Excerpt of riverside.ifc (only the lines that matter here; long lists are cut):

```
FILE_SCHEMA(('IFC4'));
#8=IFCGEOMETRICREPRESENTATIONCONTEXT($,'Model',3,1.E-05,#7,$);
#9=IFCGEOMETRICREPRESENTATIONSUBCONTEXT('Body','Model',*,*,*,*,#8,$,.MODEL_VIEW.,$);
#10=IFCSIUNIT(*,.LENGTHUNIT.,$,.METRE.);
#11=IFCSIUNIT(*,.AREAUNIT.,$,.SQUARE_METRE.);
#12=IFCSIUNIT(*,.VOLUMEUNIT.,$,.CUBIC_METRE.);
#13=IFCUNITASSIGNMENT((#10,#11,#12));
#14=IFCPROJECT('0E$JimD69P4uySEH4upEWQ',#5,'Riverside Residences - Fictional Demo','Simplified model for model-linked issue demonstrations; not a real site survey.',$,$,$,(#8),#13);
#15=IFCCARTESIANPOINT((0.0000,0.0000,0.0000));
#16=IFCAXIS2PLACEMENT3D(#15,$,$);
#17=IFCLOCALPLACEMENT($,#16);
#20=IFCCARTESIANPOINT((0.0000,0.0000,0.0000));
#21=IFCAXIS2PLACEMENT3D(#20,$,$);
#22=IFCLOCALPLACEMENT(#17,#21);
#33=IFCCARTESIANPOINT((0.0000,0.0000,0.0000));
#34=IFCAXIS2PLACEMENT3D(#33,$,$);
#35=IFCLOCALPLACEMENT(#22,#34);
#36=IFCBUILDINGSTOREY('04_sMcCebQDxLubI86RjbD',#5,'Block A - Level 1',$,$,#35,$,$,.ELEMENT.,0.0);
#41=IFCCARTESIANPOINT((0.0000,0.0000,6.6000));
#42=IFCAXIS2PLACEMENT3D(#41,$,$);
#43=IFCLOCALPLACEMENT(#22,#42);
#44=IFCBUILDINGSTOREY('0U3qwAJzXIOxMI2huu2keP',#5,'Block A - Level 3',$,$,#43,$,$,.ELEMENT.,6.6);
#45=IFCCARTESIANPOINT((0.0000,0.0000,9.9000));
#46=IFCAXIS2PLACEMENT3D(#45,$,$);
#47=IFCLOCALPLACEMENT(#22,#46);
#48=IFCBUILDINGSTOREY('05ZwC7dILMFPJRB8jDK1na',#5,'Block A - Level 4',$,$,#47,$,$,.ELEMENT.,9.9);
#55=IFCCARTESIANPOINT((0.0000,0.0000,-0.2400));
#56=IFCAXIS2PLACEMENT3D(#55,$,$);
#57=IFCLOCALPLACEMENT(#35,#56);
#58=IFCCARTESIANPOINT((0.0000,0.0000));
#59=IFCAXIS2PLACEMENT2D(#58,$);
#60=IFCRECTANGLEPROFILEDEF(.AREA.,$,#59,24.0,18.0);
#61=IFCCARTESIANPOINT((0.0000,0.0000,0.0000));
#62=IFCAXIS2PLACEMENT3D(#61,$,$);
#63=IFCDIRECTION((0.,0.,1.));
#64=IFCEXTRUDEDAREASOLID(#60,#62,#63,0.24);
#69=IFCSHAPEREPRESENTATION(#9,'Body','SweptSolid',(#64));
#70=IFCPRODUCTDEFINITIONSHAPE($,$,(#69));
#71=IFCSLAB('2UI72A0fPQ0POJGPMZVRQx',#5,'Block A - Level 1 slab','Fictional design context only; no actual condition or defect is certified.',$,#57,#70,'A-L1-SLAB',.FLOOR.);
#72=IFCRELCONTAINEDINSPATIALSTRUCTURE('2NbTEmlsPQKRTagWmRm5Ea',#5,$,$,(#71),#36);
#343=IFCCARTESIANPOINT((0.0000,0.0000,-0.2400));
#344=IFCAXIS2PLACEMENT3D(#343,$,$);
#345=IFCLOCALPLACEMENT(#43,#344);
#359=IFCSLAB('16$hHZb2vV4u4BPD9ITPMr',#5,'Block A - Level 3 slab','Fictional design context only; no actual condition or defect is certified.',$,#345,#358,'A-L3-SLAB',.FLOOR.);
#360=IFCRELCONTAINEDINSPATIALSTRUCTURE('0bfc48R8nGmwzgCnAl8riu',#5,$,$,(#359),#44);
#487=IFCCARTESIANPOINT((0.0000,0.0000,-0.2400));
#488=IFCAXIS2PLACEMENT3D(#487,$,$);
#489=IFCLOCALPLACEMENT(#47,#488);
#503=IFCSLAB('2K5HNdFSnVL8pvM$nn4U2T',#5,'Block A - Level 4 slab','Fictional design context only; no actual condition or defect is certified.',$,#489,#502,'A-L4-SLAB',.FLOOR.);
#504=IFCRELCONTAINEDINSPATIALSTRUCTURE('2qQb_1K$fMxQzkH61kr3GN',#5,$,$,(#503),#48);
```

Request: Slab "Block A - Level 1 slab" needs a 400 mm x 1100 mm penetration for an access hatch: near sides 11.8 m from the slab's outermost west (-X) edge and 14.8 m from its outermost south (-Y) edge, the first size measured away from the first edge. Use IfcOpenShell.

```python
import numpy as np
import ifcopenshell
import ifcopenshell.api.feature
import ifcopenshell.api.geometry
import ifcopenshell.api.root
import ifcopenshell.geom
import ifcopenshell.util.placement
import ifcopenshell.util.representation
import ifcopenshell.util.shape
import ifcopenshell.util.unit

model = ifcopenshell.open("riverside.ifc")
unit_scale = ifcopenshell.util.unit.calculate_unit_scale(model)
settings = ifcopenshell.geom.settings()


def volume(element):
    """Net volume in cubic metres, openings subtracted."""
    shape = ifcopenshell.geom.create_shape(settings, element)
    return ifcopenshell.util.shape.get_volume(shape.geometry)


slab = model.by_guid("2UI72A0fPQ0POJGPMZVRQx")
before = volume(slab)

# Extent in the slab's own axes, in metres. The edges named are its -X and -Y sides.
slab_shape = ifcopenshell.geom.create_shape(settings, slab)
vertices = ifcopenshell.util.shape.get_vertices(slab_shape.geometry)
x_min, y_min, bottom = vertices.min(axis=0)
top = vertices[:, 2].max()

opening = ifcopenshell.api.root.create_entity(model, ifc_class="IfcOpeningElement", name="Access hatch opening", predefined_type="OPENING")
context = ifcopenshell.util.representation.get_context(model, "Model", "Body", "MODEL_VIEW")
width, depth = 0.4, 1.1
outline = [(0.0, 0.0), (width, 0.0), (width, depth), (0.0, depth), (0.0, 0.0)]
# Overshoot both faces by 50 mm so the cut is clean.
shape = ifcopenshell.api.geometry.add_slab_representation(
    model, context=context, depth=top - bottom + 0.1, polyline=outline
)
ifcopenshell.api.geometry.assign_representation(model, product=opening, representation=shape)

matrix = ifcopenshell.util.placement.get_local_placement(slab.ObjectPlacement)
matrix[:, 3] = matrix @ np.append(np.array([x_min + 11.8, y_min + 14.8, bottom - 0.05]) / unit_scale, 1.0)
ifcopenshell.api.geometry.edit_object_placement(model, product=opening, matrix=matrix, is_si=False)
ifcopenshell.api.feature.add_feature(model, feature=opening, element=slab)

after = volume(slab)

print(f"slab volume {before:.3f} -> {after:.3f} m3")

model.write("riverside_edited.ifc")
```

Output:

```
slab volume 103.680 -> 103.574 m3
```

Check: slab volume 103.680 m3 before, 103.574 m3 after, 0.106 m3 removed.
